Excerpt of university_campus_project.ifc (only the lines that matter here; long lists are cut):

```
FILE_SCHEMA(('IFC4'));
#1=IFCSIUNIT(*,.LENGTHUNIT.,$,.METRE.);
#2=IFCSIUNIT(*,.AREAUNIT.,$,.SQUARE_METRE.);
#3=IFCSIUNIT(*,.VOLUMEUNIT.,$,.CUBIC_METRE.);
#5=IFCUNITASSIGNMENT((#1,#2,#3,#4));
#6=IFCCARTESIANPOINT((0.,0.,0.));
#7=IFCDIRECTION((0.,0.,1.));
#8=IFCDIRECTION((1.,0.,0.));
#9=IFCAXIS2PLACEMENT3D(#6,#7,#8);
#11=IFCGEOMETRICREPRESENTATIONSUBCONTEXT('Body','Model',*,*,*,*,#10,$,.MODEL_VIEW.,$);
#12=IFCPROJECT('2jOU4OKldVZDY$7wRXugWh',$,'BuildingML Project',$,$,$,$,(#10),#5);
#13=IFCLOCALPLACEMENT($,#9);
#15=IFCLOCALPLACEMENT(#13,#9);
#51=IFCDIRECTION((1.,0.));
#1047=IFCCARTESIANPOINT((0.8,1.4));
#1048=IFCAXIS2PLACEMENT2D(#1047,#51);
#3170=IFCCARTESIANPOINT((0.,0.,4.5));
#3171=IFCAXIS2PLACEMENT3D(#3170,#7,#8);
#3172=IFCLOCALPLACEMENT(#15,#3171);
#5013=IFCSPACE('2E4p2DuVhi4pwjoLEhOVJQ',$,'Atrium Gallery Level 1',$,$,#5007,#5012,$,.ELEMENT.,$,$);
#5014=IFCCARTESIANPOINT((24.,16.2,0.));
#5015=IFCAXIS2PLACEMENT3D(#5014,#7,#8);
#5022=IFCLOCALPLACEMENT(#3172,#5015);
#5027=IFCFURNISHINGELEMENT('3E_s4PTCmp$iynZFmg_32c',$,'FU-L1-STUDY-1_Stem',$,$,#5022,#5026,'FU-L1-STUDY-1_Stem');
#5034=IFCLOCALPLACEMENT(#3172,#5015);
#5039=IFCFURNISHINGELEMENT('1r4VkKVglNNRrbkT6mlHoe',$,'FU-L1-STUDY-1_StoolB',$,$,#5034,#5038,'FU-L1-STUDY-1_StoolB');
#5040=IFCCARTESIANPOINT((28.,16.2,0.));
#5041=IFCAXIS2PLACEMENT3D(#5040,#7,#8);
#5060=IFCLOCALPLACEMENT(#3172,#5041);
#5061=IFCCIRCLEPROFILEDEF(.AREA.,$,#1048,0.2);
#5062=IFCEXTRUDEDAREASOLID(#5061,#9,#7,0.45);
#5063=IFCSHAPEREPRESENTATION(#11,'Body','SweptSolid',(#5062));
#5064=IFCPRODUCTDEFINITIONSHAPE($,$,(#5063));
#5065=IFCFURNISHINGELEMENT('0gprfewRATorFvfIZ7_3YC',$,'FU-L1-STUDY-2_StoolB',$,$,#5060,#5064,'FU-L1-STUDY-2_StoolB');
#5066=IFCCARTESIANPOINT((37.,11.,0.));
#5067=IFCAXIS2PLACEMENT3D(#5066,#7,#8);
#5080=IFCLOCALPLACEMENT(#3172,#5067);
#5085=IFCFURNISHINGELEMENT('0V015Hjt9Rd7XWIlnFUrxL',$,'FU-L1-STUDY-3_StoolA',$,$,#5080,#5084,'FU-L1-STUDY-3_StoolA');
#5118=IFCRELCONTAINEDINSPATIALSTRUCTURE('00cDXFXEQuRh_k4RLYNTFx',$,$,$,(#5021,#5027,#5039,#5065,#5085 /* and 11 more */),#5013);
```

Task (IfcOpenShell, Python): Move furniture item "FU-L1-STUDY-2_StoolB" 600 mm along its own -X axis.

```python
import ifcopenshell
import ifcopenshell.api.geometry
import ifcopenshell.util.placement
import ifcopenshell.util.unit

model = ifcopenshell.open("university_campus_project.ifc")
unit_scale = ifcopenshell.util.unit.calculate_unit_scale(model)

item = model.by_id(5065)
matrix = ifcopenshell.util.placement.get_local_placement(item.ObjectPlacement)
matrix[:3, 3] -= matrix[:3, 0] * 0.6 / unit_scale
ifcopenshell.api.geometry.edit_object_placement(model, product=item, matrix=matrix, is_si=False)

print(ifcopenshell.util.placement.get_local_placement(item.ObjectPlacement).round(3) + 0.0)

model.write("university_campus_project_edited.ifc")
```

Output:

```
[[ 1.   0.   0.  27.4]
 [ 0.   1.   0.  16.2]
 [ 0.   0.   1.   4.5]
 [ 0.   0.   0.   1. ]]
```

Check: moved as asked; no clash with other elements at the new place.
